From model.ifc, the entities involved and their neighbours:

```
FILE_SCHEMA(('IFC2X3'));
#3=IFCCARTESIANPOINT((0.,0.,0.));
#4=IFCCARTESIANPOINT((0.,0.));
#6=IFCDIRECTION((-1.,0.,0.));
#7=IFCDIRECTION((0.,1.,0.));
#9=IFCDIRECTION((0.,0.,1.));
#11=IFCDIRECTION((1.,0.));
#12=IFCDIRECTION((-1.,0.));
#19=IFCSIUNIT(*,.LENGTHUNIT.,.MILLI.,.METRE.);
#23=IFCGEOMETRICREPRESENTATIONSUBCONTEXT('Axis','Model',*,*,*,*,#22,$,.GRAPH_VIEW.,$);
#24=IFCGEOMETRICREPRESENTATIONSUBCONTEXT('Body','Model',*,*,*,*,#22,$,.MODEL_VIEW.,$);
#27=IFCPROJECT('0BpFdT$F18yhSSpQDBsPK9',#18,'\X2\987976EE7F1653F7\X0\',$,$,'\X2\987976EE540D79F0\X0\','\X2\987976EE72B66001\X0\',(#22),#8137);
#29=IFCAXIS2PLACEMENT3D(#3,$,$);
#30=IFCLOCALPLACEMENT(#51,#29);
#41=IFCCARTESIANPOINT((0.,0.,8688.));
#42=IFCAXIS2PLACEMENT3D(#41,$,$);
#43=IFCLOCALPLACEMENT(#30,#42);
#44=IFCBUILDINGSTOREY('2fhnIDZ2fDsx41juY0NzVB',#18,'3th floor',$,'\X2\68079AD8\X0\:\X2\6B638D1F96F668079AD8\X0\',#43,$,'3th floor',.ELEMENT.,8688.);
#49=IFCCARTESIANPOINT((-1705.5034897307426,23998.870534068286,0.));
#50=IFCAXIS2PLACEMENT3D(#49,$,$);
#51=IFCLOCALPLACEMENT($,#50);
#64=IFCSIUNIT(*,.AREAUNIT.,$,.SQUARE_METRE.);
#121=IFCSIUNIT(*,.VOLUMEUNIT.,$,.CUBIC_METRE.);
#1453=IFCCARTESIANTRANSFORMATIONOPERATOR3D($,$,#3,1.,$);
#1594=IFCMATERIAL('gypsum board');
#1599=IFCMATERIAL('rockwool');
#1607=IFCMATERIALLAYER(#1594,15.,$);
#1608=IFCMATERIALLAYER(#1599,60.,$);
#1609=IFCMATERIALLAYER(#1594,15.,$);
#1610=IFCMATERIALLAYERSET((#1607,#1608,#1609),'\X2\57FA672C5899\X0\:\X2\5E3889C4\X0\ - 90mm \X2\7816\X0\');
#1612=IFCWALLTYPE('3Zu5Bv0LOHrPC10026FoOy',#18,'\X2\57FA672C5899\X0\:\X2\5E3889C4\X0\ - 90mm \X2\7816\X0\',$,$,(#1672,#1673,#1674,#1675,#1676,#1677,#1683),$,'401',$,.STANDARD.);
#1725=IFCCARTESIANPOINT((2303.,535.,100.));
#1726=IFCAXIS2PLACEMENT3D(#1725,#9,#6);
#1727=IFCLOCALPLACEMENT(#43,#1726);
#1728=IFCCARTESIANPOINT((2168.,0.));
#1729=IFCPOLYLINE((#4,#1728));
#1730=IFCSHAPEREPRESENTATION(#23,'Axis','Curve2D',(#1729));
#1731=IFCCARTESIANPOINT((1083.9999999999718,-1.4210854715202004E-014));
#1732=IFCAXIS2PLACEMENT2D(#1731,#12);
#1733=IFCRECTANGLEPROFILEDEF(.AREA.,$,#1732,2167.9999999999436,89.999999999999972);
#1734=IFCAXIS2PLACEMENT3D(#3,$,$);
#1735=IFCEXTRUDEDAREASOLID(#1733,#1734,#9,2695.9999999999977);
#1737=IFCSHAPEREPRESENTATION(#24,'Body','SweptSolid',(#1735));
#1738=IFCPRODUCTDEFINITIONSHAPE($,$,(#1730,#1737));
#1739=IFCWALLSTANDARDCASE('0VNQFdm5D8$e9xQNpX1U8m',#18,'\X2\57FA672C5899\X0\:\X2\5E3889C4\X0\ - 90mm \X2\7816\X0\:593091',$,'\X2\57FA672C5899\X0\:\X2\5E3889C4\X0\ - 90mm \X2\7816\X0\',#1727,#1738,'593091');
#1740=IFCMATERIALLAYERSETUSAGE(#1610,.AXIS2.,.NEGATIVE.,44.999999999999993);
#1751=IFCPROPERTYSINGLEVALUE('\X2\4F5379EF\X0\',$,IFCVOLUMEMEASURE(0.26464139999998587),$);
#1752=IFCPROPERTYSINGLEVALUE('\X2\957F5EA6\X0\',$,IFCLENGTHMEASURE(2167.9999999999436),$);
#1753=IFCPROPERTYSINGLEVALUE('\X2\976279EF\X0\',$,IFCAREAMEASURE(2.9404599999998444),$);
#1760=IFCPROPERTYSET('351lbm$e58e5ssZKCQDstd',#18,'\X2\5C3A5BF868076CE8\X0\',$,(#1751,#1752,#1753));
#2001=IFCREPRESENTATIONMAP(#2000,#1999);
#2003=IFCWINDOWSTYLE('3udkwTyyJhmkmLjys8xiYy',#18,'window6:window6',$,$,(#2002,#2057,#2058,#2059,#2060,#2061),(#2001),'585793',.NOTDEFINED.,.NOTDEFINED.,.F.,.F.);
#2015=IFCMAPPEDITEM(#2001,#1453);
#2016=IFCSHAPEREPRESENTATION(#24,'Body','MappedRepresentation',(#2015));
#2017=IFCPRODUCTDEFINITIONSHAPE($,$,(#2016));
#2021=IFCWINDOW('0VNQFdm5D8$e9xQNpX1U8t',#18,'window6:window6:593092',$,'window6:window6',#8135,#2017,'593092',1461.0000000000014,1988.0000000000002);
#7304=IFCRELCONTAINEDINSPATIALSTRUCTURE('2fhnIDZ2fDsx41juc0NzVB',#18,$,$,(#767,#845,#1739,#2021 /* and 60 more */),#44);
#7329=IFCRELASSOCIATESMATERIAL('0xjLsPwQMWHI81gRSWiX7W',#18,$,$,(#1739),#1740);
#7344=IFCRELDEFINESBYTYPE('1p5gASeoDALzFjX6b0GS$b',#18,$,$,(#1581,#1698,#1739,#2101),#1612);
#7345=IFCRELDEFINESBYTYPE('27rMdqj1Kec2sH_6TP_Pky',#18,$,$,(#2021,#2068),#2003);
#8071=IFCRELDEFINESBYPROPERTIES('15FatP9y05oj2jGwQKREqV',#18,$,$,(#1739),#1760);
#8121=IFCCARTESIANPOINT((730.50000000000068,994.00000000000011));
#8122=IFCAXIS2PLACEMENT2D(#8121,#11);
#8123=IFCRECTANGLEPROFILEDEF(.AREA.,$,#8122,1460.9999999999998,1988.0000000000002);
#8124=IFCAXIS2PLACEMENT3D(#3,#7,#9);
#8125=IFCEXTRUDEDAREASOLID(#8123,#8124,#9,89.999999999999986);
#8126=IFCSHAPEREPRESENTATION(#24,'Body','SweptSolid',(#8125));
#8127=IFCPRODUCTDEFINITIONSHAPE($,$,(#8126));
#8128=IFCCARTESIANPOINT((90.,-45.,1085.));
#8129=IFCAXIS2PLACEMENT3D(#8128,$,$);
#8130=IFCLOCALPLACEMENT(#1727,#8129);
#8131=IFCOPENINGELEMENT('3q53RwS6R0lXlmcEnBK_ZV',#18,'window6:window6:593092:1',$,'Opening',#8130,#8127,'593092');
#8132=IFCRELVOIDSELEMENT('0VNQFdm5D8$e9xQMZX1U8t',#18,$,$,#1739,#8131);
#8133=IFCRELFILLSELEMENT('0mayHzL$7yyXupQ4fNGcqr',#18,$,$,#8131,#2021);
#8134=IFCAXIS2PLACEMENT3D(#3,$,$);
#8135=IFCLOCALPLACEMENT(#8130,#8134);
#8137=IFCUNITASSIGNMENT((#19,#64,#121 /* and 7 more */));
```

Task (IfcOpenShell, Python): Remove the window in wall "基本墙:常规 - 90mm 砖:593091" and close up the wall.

```python
import ifcopenshell
import ifcopenshell.api.feature
import ifcopenshell.api.pset
import ifcopenshell.api.root
import ifcopenshell.geom
import ifcopenshell.util.element
import ifcopenshell.util.shape
import ifcopenshell.util.unit

model = ifcopenshell.open("model.ifc")
area_scale = ifcopenshell.util.unit.calculate_unit_scale(model, "AREAUNIT")
volume_scale = ifcopenshell.util.unit.calculate_unit_scale(model, "VOLUMEUNIT")
settings = ifcopenshell.geom.settings()


def volume(element):
    """Net volume in cubic metres, openings subtracted."""
    shape = ifcopenshell.geom.create_shape(settings, element)
    return ifcopenshell.util.shape.get_volume(shape.geometry)


window = model.by_guid("0VNQFdm5D8$e9xQNpX1U8t")
opening = window.FillsVoids[0].RelatingOpeningElement
wall = opening.VoidsElements[0].RelatingBuildingElement
before = volume(wall)

ifcopenshell.api.root.remove_product(model, product=window)
ifcopenshell.api.feature.remove_feature(model, feature=opening)

after = volume(wall)
thickness = 0.09  # wall thickness in metres

# Update the wall's stored quantities.
pset = model.by_id(ifcopenshell.util.element.get_pset(wall, "尺寸标注", should_inherit=False)["id"])
ifcopenshell.api.pset.edit_pset(model, pset=pset, properties={
    "体积": model.create_entity("IfcVolumeMeasure", after / volume_scale),
    "面积": model.create_entity("IfcAreaMeasure", after / thickness / area_scale),
})

print(f"wall volume {before:.3f} -> {after:.3f} m3")

model.write("model_edited.ifc")
```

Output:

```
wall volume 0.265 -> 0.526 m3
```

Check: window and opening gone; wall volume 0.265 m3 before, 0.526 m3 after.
